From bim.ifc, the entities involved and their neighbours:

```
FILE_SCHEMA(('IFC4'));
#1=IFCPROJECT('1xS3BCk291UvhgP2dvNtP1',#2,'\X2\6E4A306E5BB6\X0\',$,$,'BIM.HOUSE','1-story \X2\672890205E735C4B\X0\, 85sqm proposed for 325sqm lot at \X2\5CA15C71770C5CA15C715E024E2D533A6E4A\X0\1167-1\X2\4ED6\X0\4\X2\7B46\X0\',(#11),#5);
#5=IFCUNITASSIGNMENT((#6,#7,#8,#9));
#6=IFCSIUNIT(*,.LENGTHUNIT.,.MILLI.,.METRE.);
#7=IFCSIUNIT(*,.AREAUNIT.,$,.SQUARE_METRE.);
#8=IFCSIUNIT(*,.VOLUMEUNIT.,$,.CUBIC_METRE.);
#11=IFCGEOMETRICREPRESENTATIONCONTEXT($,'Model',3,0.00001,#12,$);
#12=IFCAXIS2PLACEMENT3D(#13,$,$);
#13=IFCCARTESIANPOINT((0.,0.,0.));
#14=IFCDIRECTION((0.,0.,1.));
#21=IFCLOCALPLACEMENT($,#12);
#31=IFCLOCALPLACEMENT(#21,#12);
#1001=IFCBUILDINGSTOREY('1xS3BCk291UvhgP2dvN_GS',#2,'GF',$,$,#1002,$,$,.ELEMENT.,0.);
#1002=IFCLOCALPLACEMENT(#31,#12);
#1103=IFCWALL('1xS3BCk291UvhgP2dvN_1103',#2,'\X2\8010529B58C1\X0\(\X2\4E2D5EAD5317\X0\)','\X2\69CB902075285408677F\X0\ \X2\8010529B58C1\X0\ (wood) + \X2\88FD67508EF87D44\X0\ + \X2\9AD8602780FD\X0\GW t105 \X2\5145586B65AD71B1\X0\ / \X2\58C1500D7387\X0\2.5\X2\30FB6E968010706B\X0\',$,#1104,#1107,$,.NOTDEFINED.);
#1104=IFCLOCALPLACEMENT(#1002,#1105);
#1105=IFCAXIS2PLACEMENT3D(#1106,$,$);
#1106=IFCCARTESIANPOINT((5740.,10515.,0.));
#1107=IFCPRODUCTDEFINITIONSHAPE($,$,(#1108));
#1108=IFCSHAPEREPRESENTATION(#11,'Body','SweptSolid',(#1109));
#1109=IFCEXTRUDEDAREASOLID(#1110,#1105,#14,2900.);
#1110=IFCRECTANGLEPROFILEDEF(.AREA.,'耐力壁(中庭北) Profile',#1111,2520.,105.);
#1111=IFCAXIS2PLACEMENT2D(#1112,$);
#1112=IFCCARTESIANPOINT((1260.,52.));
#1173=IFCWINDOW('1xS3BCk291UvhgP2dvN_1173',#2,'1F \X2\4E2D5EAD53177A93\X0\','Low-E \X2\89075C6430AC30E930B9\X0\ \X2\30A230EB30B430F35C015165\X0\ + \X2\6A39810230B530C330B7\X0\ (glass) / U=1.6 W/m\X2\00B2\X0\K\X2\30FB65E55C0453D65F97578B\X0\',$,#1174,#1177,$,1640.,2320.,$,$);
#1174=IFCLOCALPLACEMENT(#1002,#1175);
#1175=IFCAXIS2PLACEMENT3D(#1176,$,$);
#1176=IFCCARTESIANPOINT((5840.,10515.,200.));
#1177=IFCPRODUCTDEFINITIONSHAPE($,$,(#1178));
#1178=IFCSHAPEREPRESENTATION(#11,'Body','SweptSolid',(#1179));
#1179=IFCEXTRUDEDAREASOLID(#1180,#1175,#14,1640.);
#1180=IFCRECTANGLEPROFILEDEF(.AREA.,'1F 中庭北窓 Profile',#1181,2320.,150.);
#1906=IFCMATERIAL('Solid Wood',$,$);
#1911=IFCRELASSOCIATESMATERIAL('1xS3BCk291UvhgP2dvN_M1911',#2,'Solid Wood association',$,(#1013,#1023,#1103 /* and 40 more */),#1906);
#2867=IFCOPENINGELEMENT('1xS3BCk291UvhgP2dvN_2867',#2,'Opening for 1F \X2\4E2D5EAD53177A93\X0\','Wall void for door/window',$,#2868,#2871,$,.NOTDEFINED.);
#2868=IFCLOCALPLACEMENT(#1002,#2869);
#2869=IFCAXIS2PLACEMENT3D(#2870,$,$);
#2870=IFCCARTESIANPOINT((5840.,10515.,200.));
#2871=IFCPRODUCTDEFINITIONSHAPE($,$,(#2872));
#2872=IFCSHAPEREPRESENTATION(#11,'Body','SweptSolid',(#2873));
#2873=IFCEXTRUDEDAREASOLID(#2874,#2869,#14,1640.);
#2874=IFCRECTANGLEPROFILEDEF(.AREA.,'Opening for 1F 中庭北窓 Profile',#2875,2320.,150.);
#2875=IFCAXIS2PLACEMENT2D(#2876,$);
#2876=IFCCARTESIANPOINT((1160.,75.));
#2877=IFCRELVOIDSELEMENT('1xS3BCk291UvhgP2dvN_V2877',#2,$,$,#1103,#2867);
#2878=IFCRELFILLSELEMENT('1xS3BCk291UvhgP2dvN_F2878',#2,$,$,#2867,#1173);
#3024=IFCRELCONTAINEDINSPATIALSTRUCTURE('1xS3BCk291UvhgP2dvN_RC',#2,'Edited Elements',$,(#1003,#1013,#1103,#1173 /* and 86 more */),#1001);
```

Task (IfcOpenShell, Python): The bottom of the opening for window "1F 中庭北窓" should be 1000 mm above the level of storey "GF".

```python
import numpy as np
import ifcopenshell
import ifcopenshell.api.geometry
import ifcopenshell.geom
import ifcopenshell.util.element
import ifcopenshell.util.placement
import ifcopenshell.util.shape
import ifcopenshell.util.unit

model = ifcopenshell.open("bim.ifc")
unit_scale = ifcopenshell.util.unit.calculate_unit_scale(model)

window = model.by_guid("1xS3BCk291UvhgP2dvN_1173")
opening = window.FillsVoids[0].RelatingOpeningElement
storey = ifcopenshell.util.element.get_container(window, ifc_class="IfcBuildingStorey")
level = ifcopenshell.util.placement.get_local_placement(storey.ObjectPlacement)[2, 3]

# The opening's origin need not be at the sill, so measure its lowest point.
shape = ifcopenshell.geom.create_shape(ifcopenshell.geom.settings(), opening)
bottom = ifcopenshell.util.shape.get_shape_bottom_elevation(shape, shape.geometry) / unit_scale
dz = level + 1 / unit_scale - bottom

shift = np.array([0.0, 0.0, dz])
# The window is not placed relative to its opening, so move both.
for product in (opening, window):
    matrix = ifcopenshell.util.placement.get_local_placement(product.ObjectPlacement)
    matrix[:3, 3] += shift
    ifcopenshell.api.geometry.edit_object_placement(model, product=product, matrix=matrix, is_si=False)

print(f"moved by {dz * unit_scale:+.3f} m")

model.write("bim-out.ifc")
```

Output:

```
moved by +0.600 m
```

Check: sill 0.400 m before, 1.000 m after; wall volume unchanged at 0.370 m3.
